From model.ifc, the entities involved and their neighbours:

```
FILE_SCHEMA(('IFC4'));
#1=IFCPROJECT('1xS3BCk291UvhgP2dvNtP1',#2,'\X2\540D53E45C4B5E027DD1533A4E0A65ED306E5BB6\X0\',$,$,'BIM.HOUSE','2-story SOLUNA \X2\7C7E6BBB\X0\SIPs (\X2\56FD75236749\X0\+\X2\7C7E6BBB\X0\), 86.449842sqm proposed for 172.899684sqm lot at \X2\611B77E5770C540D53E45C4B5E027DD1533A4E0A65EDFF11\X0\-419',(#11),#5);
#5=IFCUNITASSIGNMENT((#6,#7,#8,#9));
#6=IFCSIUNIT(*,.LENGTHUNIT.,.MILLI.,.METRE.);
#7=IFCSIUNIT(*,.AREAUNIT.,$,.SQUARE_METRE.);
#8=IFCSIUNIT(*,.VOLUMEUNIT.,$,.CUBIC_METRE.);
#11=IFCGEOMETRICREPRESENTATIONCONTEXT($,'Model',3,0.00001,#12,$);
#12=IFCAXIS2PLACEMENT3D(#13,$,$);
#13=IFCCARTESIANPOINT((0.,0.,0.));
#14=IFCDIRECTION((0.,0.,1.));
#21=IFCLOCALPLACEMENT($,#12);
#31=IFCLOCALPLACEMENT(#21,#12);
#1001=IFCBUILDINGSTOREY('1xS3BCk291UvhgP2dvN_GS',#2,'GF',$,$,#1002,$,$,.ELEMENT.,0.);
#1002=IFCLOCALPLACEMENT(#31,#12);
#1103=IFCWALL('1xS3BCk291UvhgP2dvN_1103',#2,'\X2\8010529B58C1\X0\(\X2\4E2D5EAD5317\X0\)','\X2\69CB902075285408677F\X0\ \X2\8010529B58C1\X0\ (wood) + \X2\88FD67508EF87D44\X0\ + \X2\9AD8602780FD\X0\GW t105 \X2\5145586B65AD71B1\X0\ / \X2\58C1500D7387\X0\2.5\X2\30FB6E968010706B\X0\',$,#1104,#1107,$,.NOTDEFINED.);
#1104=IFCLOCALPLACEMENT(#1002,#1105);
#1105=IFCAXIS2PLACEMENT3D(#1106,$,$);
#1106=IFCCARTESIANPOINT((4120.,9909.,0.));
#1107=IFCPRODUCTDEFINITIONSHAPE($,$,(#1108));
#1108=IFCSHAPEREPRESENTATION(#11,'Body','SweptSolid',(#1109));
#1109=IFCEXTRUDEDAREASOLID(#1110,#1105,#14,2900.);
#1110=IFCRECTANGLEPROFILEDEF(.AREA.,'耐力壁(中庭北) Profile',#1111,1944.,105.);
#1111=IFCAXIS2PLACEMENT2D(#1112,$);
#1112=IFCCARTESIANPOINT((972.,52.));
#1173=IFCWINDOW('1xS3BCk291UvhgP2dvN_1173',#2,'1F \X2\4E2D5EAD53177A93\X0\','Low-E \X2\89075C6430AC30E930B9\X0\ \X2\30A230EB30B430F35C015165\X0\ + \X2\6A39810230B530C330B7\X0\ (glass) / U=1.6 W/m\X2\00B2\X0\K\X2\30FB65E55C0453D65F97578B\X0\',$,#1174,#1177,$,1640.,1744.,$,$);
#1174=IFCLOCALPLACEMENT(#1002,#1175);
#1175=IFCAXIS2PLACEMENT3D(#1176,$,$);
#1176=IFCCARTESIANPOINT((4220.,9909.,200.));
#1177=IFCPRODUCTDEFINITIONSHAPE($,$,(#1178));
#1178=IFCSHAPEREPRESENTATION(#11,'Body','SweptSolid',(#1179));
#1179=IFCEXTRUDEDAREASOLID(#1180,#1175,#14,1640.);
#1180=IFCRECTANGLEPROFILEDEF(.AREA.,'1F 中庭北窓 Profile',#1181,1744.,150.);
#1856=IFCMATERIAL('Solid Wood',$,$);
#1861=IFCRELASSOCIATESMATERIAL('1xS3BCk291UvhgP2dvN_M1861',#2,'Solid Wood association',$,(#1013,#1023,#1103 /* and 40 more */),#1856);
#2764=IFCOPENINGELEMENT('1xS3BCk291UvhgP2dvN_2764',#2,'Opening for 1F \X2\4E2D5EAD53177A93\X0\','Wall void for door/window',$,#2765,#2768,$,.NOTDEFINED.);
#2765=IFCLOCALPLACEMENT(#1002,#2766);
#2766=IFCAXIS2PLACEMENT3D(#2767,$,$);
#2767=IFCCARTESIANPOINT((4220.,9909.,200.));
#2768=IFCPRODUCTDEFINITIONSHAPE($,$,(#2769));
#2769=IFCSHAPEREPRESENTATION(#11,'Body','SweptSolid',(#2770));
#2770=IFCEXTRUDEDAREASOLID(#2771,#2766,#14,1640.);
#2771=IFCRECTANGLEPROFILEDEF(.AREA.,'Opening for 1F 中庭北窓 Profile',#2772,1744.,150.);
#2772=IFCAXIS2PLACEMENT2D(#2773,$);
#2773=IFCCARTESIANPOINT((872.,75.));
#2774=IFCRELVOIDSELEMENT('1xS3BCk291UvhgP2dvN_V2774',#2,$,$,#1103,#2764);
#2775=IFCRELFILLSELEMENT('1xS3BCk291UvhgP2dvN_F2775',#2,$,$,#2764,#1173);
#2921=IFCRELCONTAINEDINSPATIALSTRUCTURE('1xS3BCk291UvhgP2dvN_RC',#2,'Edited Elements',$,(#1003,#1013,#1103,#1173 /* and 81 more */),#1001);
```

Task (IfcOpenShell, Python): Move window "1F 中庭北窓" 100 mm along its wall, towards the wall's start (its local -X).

```python
import ifcopenshell
import ifcopenshell.api.geometry
import ifcopenshell.util.placement

model = ifcopenshell.open("model.ifc")

window = model.by_guid("1xS3BCk291UvhgP2dvN_1173")
opening = window.FillsVoids[0].RelatingOpeningElement
wall = opening.VoidsElements[0].RelatingBuildingElement

wall_matrix = ifcopenshell.util.placement.get_local_placement(wall.ObjectPlacement)
shift = wall_matrix[:3, 0] * -100.0
before = ifcopenshell.util.placement.get_local_placement(window.ObjectPlacement)[:3, 3].copy()

# The window is not placed relative to its opening, so move both.
for product in (opening, window):
    matrix = ifcopenshell.util.placement.get_local_placement(product.ObjectPlacement)
    matrix[:3, 3] += shift
    ifcopenshell.api.geometry.edit_object_placement(model, product=product, matrix=matrix, is_si=False)

after = ifcopenshell.util.placement.get_local_placement(window.ObjectPlacement)[:3, 3]
print("window moved by", (after - before).round(3) + 0.0)

model.write("model-out.ifc")
```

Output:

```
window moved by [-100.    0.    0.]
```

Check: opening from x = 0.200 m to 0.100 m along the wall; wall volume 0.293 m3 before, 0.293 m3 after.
